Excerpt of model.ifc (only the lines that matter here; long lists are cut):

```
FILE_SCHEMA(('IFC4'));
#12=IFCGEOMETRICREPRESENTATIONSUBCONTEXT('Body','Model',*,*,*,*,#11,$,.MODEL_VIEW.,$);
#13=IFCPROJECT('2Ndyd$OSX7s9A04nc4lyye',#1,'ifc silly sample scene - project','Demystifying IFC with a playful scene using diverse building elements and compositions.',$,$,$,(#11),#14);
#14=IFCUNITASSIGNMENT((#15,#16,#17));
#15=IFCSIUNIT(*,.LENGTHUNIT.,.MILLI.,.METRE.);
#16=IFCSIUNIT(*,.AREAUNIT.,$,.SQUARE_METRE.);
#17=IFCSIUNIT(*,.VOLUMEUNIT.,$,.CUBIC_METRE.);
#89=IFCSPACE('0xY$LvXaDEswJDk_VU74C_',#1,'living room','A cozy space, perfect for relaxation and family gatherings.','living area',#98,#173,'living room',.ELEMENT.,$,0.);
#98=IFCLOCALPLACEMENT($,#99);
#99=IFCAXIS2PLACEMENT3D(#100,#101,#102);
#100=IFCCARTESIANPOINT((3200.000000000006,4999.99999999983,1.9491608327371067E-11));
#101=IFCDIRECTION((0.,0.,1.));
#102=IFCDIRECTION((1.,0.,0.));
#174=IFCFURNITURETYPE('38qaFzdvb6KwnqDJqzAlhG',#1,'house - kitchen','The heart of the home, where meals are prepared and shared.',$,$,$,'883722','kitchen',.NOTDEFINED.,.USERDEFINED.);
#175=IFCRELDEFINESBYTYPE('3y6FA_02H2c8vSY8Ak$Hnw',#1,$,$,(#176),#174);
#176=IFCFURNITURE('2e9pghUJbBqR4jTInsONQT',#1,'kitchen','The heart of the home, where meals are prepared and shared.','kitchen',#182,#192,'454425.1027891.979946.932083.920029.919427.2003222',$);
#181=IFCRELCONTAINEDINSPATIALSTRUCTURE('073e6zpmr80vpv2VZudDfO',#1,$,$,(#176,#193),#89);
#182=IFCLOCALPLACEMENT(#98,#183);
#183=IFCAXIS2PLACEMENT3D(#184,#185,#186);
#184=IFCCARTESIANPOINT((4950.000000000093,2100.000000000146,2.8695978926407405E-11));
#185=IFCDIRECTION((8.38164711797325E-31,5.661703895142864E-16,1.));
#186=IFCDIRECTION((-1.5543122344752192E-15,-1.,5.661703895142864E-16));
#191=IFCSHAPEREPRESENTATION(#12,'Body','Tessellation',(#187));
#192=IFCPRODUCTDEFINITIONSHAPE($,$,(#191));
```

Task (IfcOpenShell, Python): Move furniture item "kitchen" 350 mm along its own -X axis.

```python
import ifcopenshell
import ifcopenshell.api.geometry
import ifcopenshell.util.placement
import ifcopenshell.util.unit

model = ifcopenshell.open("model.ifc")
unit_scale = ifcopenshell.util.unit.calculate_unit_scale(model)

item = model.by_id(176)
matrix = ifcopenshell.util.placement.get_local_placement(item.ObjectPlacement)
matrix[:3, 3] -= matrix[:3, 0] * 0.35 / unit_scale
ifcopenshell.api.geometry.edit_object_placement(model, product=item, matrix=matrix, is_si=False)

print(ifcopenshell.util.placement.get_local_placement(item.ObjectPlacement).round(3) + 0.0)

model.write("model_updated.ifc")
```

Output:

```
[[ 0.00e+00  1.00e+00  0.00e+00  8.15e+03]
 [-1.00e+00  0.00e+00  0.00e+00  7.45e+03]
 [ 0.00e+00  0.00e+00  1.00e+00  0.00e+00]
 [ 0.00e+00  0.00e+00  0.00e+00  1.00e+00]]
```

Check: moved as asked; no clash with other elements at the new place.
